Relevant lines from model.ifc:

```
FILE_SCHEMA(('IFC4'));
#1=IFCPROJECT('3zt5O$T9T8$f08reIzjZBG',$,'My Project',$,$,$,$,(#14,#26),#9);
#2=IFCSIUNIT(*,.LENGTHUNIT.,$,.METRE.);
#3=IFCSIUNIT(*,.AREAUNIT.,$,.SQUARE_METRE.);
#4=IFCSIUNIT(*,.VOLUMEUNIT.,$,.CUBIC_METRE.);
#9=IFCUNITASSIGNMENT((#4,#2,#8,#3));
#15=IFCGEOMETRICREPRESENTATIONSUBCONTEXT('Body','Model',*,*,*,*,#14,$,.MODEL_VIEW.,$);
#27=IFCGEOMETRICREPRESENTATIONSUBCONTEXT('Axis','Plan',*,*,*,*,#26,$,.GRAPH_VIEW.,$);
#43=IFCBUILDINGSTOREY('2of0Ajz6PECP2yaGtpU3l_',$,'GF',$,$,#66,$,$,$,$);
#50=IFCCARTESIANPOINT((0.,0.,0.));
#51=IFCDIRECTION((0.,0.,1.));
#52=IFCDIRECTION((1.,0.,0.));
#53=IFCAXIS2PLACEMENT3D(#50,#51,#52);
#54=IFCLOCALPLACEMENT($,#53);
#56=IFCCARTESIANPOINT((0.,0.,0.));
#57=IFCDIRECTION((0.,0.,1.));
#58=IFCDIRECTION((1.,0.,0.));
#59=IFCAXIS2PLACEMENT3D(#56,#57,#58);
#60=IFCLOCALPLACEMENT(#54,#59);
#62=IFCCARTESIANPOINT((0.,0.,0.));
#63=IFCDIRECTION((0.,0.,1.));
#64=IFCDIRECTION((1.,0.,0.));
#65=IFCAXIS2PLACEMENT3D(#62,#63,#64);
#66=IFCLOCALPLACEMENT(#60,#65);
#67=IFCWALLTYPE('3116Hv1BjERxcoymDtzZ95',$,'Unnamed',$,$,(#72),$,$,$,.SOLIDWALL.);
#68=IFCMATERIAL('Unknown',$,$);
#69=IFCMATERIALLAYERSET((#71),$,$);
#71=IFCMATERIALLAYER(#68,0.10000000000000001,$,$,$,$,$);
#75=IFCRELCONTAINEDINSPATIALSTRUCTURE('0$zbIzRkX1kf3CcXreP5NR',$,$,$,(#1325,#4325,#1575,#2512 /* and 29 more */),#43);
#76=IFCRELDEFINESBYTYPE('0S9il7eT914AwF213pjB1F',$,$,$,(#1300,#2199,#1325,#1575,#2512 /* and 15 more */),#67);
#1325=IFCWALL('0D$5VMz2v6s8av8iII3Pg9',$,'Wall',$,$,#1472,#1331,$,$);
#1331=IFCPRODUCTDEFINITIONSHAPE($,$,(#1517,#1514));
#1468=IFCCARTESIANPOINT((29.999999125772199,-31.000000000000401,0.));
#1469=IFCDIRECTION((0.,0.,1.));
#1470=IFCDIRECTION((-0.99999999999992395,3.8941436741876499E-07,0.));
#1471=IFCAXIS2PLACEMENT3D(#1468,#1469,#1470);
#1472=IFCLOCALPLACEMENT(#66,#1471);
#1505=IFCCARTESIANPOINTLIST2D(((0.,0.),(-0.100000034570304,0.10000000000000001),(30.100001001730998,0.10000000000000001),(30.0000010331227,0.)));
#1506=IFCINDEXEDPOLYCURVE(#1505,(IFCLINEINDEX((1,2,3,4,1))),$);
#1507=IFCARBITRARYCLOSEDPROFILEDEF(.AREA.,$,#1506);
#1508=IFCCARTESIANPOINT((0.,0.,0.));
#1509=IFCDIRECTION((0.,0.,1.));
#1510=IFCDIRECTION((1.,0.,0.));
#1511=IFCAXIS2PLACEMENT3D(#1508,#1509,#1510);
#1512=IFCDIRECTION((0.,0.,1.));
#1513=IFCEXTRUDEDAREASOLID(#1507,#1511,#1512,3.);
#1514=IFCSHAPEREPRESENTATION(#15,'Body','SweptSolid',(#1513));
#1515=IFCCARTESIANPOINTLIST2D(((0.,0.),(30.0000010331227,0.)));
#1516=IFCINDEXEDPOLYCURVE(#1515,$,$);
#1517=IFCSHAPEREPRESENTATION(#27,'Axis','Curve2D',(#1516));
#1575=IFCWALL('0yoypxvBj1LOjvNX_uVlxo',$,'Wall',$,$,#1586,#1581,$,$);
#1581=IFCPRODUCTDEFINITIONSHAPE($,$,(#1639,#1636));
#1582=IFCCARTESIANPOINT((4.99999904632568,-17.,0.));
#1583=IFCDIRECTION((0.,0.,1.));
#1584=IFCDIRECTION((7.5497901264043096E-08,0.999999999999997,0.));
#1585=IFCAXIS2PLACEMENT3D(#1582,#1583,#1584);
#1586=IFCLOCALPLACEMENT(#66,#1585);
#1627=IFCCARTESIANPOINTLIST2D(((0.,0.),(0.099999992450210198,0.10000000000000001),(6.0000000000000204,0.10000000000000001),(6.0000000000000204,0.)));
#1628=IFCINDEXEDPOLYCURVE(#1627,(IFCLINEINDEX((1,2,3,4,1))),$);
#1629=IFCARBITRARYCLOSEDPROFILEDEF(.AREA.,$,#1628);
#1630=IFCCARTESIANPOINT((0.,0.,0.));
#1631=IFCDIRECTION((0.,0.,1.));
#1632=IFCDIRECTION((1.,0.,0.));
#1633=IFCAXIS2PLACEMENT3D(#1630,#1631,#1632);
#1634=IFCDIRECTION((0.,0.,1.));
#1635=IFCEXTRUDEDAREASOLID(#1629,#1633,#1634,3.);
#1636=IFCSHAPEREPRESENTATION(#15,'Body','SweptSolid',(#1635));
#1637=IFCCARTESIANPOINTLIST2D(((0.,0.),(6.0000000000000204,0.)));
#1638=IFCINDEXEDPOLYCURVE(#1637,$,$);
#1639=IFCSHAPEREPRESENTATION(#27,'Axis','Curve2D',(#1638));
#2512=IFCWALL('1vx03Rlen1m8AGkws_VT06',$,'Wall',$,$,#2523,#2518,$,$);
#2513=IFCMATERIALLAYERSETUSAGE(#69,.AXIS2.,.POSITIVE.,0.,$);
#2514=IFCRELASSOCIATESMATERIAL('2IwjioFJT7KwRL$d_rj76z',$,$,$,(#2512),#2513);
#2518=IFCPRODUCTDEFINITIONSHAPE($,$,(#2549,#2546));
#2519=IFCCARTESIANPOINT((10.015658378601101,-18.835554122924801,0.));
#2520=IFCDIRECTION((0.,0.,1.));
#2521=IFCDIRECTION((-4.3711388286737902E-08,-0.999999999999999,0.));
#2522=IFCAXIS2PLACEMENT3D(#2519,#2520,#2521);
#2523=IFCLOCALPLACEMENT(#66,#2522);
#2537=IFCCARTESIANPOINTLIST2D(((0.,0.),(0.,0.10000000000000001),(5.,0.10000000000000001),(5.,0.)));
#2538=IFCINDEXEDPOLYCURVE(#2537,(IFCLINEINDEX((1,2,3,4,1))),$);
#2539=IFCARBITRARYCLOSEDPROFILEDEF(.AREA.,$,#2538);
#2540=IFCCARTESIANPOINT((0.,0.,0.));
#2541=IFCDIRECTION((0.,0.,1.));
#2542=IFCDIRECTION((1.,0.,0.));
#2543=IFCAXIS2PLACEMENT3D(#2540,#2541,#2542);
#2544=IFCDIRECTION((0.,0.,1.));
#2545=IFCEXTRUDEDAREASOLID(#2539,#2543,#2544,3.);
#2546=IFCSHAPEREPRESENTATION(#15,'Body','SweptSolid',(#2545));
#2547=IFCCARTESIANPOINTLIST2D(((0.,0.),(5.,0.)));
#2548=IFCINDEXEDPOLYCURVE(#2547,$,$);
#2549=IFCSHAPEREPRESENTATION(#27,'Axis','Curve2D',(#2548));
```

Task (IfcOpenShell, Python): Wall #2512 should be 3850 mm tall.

```python
import ifcopenshell
import ifcopenshell.geom
import ifcopenshell.util.representation
import ifcopenshell.util.shape
import ifcopenshell.util.unit

model = ifcopenshell.open("model.ifc")
unit_scale = ifcopenshell.util.unit.calculate_unit_scale(model)
settings = ifcopenshell.geom.settings()


def volume(element):
    """Net volume in cubic metres, openings subtracted."""
    shape = ifcopenshell.geom.create_shape(settings, element)
    return ifcopenshell.util.shape.get_volume(shape.geometry)


wall = model.by_id(2512)
before = volume(wall)

body = ifcopenshell.util.representation.get_representation(wall, "Model", "Body")
solid = body.Items[0]
old_height = solid.Depth
solid.Depth = 3.85 / unit_scale
after = volume(wall)

print(f"height {old_height:g} -> {solid.Depth:g}, volume {before:.3f} -> {after:.3f} m3")

model.write("model_updated.ifc")
```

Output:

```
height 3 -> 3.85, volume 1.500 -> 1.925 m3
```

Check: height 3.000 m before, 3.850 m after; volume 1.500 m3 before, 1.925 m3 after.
